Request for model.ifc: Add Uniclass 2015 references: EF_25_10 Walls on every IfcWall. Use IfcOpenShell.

First a look at what the model holds.

```python
import ifcopenshell

model = ifcopenshell.open("model.ifc")
print(model.schema)
print("classifications:", [c.Name for c in model.by_type("IfcClassification")])
for ifc_class in ("IfcDoor", "IfcRoof", "IfcStair", "IfcWall", "IfcWindow"):
    print(ifc_class, len(model.by_type(ifc_class)))
```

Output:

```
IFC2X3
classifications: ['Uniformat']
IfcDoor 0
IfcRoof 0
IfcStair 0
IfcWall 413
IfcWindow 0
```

```python
import ifcopenshell
import ifcopenshell.api.classification

model = ifcopenshell.open("model.ifc")

# IFC2X3 requires Source and Edition and has no link from the project to the system.
system = model.create_entity("IfcClassification", Source="NBS", Edition="2015", Name="Uniclass 2015")

codes = {
    "IfcWall": ("EF_25_10", "Walls"),
}
for ifc_class, (code, name) in codes.items():
    products = model.by_type(ifc_class)
    ifcopenshell.api.classification.add_reference(
        model, products=products, classification=system, identification=code, name=name
    )
    print(code, len(products))

model.write("model_edited.ifc")
```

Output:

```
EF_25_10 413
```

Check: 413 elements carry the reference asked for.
